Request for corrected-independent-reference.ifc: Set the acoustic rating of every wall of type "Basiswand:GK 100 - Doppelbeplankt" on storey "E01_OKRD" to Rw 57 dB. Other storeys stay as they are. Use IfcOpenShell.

First a look at what the model holds.

```python
import ifcopenshell
import ifcopenshell.util.element

model = ifcopenshell.open("corrected-independent-reference.ifc")
print(model.schema)
storey = next(s for s in model.by_type("IfcBuildingStorey") if s.Name == "E01_OKRD")
walls = [e for e in ifcopenshell.util.element.get_decomposition(storey) if e.is_a("IfcWall")]
seen = {}
for e in walls:
    element_type = ifcopenshell.util.element.get_type(e)
    key = (element_type.Name if element_type != e and element_type else None, ifcopenshell.util.element.get_pset(e, "Pset_WallCommon", "AcousticRating"))
    seen[key] = seen.get(key, 0) + 1
for (name, value), count in sorted(seen.items(), key=str):
    print(count, "x", name, "|", value)
```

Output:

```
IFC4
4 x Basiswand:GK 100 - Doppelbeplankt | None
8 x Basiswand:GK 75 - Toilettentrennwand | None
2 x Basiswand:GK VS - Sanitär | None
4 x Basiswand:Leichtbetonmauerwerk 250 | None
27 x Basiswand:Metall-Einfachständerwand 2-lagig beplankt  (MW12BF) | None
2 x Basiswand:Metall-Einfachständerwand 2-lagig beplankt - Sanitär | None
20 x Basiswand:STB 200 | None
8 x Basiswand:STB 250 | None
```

```python
import ifcopenshell
import ifcopenshell.api.pset
import ifcopenshell.util.element

model = ifcopenshell.open("corrected-independent-reference.ifc")

storey = next(s for s in model.by_type("IfcBuildingStorey") if s.Name == "E01_OKRD")
walls = [e for e in ifcopenshell.util.element.get_decomposition(storey) if e.is_a("IfcWall")]

count = 0
for e in walls:
    element_type = ifcopenshell.util.element.get_type(e)
    if element_type in (None, e) or element_type.Name != "Basiswand:GK 100 - Doppelbeplankt":
        continue
    # add_pset returns the element's existing set when there is one.
    pset = ifcopenshell.api.pset.add_pset(model, product=e, name="Pset_WallCommon")
    ifcopenshell.api.pset.edit_pset(model, pset=pset, properties={"AcousticRating": "Rw 57 dB"})
    count += 1

print(count, "walls updated")

model.write("corrected-independent-reference_edited.ifc")
```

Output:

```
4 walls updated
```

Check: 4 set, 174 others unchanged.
